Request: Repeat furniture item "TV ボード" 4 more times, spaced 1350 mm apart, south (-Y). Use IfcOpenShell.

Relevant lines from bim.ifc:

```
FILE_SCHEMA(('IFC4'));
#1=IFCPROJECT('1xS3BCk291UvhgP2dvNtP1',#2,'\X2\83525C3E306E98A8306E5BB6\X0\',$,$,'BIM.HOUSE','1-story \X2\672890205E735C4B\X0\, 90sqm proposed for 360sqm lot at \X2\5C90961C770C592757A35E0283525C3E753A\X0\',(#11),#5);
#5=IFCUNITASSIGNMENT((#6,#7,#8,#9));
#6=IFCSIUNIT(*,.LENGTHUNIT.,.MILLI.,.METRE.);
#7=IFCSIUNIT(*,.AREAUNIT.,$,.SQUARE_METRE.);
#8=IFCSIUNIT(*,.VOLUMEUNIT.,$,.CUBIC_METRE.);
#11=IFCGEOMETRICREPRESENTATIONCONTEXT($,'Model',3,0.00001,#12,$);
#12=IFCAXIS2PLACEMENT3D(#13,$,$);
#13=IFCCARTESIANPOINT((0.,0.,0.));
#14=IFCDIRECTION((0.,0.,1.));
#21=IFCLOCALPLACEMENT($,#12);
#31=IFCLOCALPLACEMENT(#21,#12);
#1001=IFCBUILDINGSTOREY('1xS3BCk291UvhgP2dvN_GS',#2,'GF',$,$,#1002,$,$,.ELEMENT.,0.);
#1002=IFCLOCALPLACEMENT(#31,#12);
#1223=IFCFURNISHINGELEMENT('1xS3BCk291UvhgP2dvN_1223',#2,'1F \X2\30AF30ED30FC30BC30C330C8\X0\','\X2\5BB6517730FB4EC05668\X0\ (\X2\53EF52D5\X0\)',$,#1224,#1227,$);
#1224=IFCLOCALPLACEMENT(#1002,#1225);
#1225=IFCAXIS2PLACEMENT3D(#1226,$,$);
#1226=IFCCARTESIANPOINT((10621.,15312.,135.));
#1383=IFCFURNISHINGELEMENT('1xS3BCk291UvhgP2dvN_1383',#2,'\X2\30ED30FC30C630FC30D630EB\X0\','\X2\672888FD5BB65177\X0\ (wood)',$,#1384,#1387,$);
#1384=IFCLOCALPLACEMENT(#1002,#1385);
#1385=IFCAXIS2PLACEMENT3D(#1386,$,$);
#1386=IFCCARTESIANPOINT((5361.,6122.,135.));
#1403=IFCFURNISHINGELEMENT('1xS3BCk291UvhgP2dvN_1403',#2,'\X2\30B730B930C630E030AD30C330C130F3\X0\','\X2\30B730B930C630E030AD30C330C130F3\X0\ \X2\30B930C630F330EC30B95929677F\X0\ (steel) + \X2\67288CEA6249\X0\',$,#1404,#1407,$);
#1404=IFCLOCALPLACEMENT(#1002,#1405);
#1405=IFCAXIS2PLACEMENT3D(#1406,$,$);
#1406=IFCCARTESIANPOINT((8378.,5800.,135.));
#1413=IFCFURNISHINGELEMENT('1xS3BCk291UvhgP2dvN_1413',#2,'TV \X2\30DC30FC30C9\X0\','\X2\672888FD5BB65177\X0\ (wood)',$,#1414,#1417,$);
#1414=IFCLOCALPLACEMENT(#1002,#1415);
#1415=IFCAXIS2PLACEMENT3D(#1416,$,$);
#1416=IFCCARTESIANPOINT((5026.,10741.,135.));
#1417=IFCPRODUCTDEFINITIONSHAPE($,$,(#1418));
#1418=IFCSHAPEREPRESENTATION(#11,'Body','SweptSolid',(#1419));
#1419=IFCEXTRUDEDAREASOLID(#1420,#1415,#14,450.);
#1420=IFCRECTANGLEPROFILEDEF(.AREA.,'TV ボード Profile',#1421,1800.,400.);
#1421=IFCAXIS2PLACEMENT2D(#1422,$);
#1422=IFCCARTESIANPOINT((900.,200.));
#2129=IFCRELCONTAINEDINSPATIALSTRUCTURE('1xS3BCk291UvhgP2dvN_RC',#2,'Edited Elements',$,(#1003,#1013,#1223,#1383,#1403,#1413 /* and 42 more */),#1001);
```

```python
import numpy as np
import ifcopenshell
import ifcopenshell.api.geometry
import ifcopenshell.api.root
import ifcopenshell.util.element
import ifcopenshell.util.placement

model = ifcopenshell.open("bim.ifc")


def reuse_history(source, copy):
    """copy_class also copies each property set's owner history, people and application; keep the originals."""
    for rel in copy.IsDefinedBy:
        if rel.is_a("IfcRelDefinesByProperties") and (history := rel.RelatingPropertyDefinition.OwnerHistory):
            rel.RelatingPropertyDefinition.OwnerHistory = source.OwnerHistory
            ifcopenshell.util.element.remove_deep2(model, history)


source = model.by_id(1413)
base = ifcopenshell.util.placement.get_local_placement(source.ObjectPlacement)
step = np.array([0.0, -1.0, 0.0]) * 1350.0

for i in range(1, 5):
    copy = ifcopenshell.api.root.copy_class(model, product=source)
    copy.Representation = ifcopenshell.util.element.copy_deep(
        model, source.Representation, exclude=["IfcGeometricRepresentationContext", "IfcRepresentationMap"]
    )
    reuse_history(source, copy)
    matrix = base.copy()
    matrix[:3, 3] += i * step
    print("added at", matrix[:3, 3].round(3) + 0.0)
    ifcopenshell.api.geometry.edit_object_placement(model, product=copy, matrix=matrix, is_si=False)

model.write("bim-out.ifc")
```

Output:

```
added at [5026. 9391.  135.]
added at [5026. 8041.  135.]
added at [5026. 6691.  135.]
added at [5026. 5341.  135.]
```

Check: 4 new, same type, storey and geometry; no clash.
